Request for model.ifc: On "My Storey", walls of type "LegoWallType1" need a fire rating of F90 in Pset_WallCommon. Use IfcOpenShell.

First a look at what the model holds.

```python
import ifcopenshell
import ifcopenshell.util.element

model = ifcopenshell.open("model.ifc")
print(model.schema)
storey = next(s for s in model.by_type("IfcBuildingStorey") if s.Name == "My Storey")
walls = [e for e in ifcopenshell.util.element.get_decomposition(storey) if e.is_a("IfcWall")]
seen = {}
for e in walls:
    element_type = ifcopenshell.util.element.get_type(e)
    key = (element_type.Name if element_type != e and element_type else None, ifcopenshell.util.element.get_pset(e, "Pset_WallCommon", "FireRating"))
    seen[key] = seen.get(key, 0) + 1
for (name, value), count in sorted(seen.items(), key=str):
    print(count, "x", name, "|", value)
```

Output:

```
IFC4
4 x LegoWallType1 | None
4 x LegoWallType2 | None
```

```python
import ifcopenshell
import ifcopenshell.api.pset
import ifcopenshell.util.element

model = ifcopenshell.open("model.ifc")

storey = next(s for s in model.by_type("IfcBuildingStorey") if s.Name == "My Storey")
walls = [e for e in ifcopenshell.util.element.get_decomposition(storey) if e.is_a("IfcWall")]

count = 0
for e in walls:
    element_type = ifcopenshell.util.element.get_type(e)
    if element_type in (None, e) or element_type.Name != "LegoWallType1":
        continue
    # add_pset returns the element's existing set when there is one.
    pset = ifcopenshell.api.pset.add_pset(model, product=e, name="Pset_WallCommon")
    ifcopenshell.api.pset.edit_pset(model, pset=pset, properties={"FireRating": "F90"})
    count += 1

print(count, "walls updated")

model.write("model-out.ifc")
```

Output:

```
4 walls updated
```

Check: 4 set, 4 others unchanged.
